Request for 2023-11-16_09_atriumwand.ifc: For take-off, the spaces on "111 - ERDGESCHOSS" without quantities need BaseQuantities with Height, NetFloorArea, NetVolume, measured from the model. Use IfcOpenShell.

First a look at what the model holds.

```python
import ifcopenshell
import ifcopenshell.util.element
import ifcopenshell.util.unit

model = ifcopenshell.open("2023-11-16_09_atriumwand.ifc")
print(model.schema)
for unit_type in ("LENGTHUNIT", "AREAUNIT", "VOLUMEUNIT"):
    print(unit_type, ifcopenshell.util.unit.calculate_unit_scale(model, unit_type))
storey = next(s for s in model.by_type("IfcBuildingStorey") if s.Name == "111 - ERDGESCHOSS")
spaces = [e for e in ifcopenshell.util.element.get_decomposition(storey) if e.is_a("IfcSpace")]
for e in sorted(spaces, key=lambda e: e.id()):
    print(e.id(), e.is_a(), e.Name, list(ifcopenshell.util.element.get_psets(e, qtos_only=True)), sep=" | ")
```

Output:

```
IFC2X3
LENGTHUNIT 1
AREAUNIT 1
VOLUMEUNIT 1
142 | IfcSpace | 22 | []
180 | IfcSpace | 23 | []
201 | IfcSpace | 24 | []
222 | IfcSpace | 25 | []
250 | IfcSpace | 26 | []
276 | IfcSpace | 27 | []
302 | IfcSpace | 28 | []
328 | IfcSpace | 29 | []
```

```python
import ifcopenshell
import ifcopenshell.api.pset
import ifcopenshell.geom
import ifcopenshell.util.element
import ifcopenshell.util.shape
import ifcopenshell.util.unit

model = ifcopenshell.open("2023-11-16_09_atriumwand.ifc")
unit_scale = ifcopenshell.util.unit.calculate_unit_scale(model)
area_scale = ifcopenshell.util.unit.calculate_unit_scale(model, "AREAUNIT")
volume_scale = ifcopenshell.util.unit.calculate_unit_scale(model, "VOLUMEUNIT")
settings = ifcopenshell.geom.settings()

storey = next(s for s in model.by_type("IfcBuildingStorey") if s.Name == "111 - ERDGESCHOSS")
spaces = [e for e in ifcopenshell.util.element.get_decomposition(storey) if e.is_a("IfcSpace")]

for e in sorted(spaces, key=lambda e: e.id()):
    if ifcopenshell.util.element.get_psets(e, qtos_only=True, should_inherit=False):
        continue
    # Geometry comes back in metres, in the element's own axes.
    shape = ifcopenshell.geom.create_shape(settings, e)
    values = {
        "Height": ifcopenshell.util.shape.get_z(shape.geometry) / unit_scale,
        "NetFloorArea": ifcopenshell.util.shape.get_footprint_area(shape.geometry) / area_scale,
        "NetVolume": ifcopenshell.util.shape.get_volume(shape.geometry) / volume_scale,
    }
    qto = ifcopenshell.api.pset.add_qto(model, product=e, name="BaseQuantities")
    ifcopenshell.api.pset.edit_qto(model, qto=qto, properties=values)
    print(e.id(), {k: round(v, 3) for k, v in values.items()})

model.write("2023-11-16_09_atriumwand_rev.ifc")
```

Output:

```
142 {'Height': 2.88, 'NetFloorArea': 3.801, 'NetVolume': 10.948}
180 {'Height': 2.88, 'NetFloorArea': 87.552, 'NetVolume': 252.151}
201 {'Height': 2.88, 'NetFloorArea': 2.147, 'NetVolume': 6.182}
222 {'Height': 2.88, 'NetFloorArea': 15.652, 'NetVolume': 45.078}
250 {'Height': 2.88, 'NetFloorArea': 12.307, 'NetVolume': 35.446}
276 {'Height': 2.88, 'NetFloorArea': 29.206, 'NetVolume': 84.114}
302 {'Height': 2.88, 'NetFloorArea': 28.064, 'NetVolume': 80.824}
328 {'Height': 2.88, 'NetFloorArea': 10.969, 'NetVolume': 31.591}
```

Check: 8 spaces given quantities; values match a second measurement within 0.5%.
